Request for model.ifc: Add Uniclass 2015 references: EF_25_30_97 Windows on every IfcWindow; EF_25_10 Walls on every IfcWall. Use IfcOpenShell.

First a look at what the model holds.

```python
import ifcopenshell

model = ifcopenshell.open("model.ifc")
print(model.schema)
print("classifications:", [c.Name for c in model.by_type("IfcClassification")])
for ifc_class in ("IfcDoor", "IfcRoof", "IfcStair", "IfcWall", "IfcWindow"):
    print(ifc_class, len(model.by_type(ifc_class)))
```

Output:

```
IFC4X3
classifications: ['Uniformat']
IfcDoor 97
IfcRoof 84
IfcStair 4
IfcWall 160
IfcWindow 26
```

```python
import ifcopenshell
import ifcopenshell.api.classification

model = ifcopenshell.open("model.ifc")

system = ifcopenshell.api.classification.add_classification(model, classification="Uniclass 2015")

codes = {
    "IfcWindow": ("EF_25_30_97", "Windows"),
    "IfcWall": ("EF_25_10", "Walls"),
}
for ifc_class, (code, name) in codes.items():
    products = model.by_type(ifc_class)
    ifcopenshell.api.classification.add_reference(
        model, products=products, classification=system, identification=code, name=name
    )
    print(code, len(products))

model.write("model_updated.ifc")
```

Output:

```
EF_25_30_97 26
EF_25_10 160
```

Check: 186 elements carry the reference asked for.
